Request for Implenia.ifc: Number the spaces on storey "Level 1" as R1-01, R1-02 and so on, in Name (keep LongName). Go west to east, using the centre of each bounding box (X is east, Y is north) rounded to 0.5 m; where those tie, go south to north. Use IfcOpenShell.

First a look at what the model holds.

```python
import ifcopenshell
import ifcopenshell.util.element
import ifcopenshell.util.placement

model = ifcopenshell.open("Implenia.ifc")
print(model.schema)
storey = next(s for s in model.by_type("IfcBuildingStorey") if s.Name == "Level 1")
spaces = [e for e in ifcopenshell.util.element.get_decomposition(storey) if e.is_a("IfcSpace")]
for e in sorted(spaces, key=lambda e: e.id()):
    origin = ifcopenshell.util.placement.get_local_placement(e.ObjectPlacement)[:3, 3]
    print(e.id(), e.Name, e.LongName, origin.round(2) + 0.0, sep=" | ")
```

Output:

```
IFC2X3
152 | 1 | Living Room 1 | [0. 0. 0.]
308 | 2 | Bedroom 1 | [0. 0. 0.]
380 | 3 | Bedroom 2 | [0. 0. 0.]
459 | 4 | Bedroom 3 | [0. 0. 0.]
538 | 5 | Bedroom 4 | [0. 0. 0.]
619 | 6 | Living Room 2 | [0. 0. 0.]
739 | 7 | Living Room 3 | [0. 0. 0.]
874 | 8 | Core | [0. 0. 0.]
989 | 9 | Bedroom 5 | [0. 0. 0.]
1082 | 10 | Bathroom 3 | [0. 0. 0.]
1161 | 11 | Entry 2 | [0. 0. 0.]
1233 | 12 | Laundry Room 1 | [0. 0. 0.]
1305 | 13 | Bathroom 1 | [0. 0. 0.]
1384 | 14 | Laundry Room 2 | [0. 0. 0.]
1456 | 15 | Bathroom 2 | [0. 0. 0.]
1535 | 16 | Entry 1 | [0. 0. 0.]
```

```python
import ifcopenshell
import ifcopenshell.geom
import ifcopenshell.util.element
import ifcopenshell.util.shape

model = ifcopenshell.open("Implenia.ifc")
settings = ifcopenshell.geom.settings()
settings.set("use-world-coords", True)


def centre(element):
    shape = ifcopenshell.geom.create_shape(settings, element)
    return ifcopenshell.util.shape.get_bbox_centroid(shape.geometry)


storey = next(s for s in model.by_type("IfcBuildingStorey") if s.Name == "Level 1")
spaces = [e for e in ifcopenshell.util.element.get_decomposition(storey) if e.is_a("IfcSpace")]

# Insertion points can sit at a corner or the storey origin, so sort by the geometry (in metres).
centres = {e: centre(e) for e in spaces}
spaces.sort(key=lambda e: (round(centres[e][0] / 0.5), centres[e][1]))

for i, e in enumerate(spaces, start=1):
    number = f"R1-{i:02d}"
    e.Name = number
    print(e.id(), number)

model.write("Implenia_updated.ifc")
```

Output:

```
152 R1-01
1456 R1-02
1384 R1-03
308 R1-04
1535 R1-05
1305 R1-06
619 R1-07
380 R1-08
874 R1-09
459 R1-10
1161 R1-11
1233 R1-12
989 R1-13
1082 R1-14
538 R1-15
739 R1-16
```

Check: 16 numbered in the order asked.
